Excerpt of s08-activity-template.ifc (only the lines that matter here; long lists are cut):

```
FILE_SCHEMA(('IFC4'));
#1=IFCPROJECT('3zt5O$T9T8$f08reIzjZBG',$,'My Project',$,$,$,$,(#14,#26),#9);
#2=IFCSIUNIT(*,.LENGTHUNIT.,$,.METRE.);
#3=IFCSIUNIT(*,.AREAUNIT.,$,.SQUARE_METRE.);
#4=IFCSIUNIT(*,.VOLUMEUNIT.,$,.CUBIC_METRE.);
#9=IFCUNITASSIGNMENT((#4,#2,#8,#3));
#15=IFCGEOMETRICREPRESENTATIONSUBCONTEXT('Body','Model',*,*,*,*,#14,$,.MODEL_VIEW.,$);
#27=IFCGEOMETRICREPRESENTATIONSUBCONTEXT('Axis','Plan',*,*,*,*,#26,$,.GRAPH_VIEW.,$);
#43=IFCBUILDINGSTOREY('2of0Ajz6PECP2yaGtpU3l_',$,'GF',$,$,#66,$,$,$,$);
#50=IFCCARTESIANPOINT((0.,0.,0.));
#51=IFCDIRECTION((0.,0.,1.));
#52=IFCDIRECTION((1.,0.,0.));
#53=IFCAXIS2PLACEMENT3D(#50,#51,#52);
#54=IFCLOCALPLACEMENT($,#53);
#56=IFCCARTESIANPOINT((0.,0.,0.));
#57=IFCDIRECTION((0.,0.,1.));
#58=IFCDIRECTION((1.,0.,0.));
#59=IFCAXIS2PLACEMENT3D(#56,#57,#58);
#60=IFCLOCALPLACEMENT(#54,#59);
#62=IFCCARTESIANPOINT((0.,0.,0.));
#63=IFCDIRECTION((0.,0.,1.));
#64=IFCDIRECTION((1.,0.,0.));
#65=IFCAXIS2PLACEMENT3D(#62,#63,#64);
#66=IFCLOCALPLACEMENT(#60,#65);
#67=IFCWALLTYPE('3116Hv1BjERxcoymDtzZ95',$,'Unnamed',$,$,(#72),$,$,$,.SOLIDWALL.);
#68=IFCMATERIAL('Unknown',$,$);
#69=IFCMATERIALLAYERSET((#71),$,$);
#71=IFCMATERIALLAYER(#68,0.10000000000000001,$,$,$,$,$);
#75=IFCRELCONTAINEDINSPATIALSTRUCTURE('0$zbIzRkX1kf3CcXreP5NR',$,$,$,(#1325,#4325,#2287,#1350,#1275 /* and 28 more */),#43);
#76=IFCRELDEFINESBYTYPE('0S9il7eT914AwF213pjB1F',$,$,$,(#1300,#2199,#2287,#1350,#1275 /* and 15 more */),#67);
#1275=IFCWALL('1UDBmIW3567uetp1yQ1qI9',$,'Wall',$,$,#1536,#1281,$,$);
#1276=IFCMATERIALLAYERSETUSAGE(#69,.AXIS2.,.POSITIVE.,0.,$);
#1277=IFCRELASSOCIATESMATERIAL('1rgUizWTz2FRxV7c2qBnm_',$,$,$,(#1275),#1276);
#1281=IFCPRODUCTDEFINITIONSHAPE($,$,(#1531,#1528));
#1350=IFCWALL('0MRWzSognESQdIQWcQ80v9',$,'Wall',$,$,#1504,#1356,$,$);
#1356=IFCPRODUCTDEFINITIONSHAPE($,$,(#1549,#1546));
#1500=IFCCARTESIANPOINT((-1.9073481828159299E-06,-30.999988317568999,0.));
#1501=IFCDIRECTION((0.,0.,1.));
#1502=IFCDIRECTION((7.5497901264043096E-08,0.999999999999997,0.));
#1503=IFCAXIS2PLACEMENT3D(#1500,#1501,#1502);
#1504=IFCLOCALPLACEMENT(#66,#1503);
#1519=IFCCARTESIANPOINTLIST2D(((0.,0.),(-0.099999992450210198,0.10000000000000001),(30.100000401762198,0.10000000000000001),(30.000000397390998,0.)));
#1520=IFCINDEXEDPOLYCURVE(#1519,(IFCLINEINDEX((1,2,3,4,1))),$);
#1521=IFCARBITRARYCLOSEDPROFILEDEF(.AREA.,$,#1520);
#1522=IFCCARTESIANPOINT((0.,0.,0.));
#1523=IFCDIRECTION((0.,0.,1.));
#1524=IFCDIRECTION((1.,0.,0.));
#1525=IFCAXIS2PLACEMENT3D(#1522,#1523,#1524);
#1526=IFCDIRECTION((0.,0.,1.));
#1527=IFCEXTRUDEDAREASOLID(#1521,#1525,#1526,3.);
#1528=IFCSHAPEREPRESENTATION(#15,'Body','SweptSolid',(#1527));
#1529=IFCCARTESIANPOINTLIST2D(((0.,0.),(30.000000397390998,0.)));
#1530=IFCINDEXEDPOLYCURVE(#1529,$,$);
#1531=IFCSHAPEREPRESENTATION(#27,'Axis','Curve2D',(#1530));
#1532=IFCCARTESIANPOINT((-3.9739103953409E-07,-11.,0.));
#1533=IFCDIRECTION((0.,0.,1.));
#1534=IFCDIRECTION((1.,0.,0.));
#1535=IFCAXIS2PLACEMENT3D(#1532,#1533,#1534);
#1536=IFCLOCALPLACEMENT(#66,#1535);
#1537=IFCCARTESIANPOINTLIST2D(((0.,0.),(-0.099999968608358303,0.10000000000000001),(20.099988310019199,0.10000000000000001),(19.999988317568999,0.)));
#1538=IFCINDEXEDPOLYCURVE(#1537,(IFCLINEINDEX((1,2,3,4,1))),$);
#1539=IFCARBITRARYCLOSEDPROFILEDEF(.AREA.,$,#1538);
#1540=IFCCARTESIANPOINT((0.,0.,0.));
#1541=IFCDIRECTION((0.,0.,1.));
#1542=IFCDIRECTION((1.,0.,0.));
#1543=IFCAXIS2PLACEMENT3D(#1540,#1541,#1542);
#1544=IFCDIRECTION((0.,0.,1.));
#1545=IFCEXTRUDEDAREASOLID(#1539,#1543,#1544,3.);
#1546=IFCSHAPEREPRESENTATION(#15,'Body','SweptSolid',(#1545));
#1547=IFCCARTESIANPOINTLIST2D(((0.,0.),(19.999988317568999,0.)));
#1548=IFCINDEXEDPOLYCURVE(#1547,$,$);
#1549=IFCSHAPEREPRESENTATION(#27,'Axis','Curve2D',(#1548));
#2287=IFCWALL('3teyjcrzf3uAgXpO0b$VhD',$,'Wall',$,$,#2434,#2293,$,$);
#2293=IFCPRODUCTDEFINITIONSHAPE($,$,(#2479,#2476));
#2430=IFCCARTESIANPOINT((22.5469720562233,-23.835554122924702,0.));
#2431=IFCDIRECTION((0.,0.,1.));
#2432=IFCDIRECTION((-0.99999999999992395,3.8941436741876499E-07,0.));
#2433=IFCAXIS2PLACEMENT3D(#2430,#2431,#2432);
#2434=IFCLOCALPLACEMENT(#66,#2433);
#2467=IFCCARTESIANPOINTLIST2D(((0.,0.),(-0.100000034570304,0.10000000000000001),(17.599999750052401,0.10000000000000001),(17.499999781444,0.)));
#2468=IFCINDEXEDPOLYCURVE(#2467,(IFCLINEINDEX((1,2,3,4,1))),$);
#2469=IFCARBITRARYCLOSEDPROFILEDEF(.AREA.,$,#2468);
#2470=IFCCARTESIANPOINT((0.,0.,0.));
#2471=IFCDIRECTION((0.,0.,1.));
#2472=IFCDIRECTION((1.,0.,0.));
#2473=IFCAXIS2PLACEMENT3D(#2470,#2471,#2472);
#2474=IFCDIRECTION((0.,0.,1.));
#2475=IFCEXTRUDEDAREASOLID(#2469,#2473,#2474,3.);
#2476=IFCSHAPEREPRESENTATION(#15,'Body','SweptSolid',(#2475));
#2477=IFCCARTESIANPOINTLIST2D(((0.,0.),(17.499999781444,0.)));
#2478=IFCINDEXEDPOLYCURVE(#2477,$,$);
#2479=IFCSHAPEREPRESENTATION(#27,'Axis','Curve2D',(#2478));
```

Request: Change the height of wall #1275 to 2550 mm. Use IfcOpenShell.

```python
import ifcopenshell
import ifcopenshell.geom
import ifcopenshell.util.representation
import ifcopenshell.util.shape
import ifcopenshell.util.unit

model = ifcopenshell.open("s08-activity-template.ifc")
unit_scale = ifcopenshell.util.unit.calculate_unit_scale(model)
settings = ifcopenshell.geom.settings()


def volume(element):
    """Net volume in cubic metres, openings subtracted."""
    shape = ifcopenshell.geom.create_shape(settings, element)
    return ifcopenshell.util.shape.get_volume(shape.geometry)


wall = model.by_id(1275)
before = volume(wall)

body = ifcopenshell.util.representation.get_representation(wall, "Model", "Body")
solid = body.Items[0]
old_height = solid.Depth
solid.Depth = 2.55 / unit_scale
after = volume(wall)

print(f"height {old_height:g} -> {solid.Depth:g}, volume {before:.3f} -> {after:.3f} m3")

model.write("s08-activity-template_edited.ifc")
```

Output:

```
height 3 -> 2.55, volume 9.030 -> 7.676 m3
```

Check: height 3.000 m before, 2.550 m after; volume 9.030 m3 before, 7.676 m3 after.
